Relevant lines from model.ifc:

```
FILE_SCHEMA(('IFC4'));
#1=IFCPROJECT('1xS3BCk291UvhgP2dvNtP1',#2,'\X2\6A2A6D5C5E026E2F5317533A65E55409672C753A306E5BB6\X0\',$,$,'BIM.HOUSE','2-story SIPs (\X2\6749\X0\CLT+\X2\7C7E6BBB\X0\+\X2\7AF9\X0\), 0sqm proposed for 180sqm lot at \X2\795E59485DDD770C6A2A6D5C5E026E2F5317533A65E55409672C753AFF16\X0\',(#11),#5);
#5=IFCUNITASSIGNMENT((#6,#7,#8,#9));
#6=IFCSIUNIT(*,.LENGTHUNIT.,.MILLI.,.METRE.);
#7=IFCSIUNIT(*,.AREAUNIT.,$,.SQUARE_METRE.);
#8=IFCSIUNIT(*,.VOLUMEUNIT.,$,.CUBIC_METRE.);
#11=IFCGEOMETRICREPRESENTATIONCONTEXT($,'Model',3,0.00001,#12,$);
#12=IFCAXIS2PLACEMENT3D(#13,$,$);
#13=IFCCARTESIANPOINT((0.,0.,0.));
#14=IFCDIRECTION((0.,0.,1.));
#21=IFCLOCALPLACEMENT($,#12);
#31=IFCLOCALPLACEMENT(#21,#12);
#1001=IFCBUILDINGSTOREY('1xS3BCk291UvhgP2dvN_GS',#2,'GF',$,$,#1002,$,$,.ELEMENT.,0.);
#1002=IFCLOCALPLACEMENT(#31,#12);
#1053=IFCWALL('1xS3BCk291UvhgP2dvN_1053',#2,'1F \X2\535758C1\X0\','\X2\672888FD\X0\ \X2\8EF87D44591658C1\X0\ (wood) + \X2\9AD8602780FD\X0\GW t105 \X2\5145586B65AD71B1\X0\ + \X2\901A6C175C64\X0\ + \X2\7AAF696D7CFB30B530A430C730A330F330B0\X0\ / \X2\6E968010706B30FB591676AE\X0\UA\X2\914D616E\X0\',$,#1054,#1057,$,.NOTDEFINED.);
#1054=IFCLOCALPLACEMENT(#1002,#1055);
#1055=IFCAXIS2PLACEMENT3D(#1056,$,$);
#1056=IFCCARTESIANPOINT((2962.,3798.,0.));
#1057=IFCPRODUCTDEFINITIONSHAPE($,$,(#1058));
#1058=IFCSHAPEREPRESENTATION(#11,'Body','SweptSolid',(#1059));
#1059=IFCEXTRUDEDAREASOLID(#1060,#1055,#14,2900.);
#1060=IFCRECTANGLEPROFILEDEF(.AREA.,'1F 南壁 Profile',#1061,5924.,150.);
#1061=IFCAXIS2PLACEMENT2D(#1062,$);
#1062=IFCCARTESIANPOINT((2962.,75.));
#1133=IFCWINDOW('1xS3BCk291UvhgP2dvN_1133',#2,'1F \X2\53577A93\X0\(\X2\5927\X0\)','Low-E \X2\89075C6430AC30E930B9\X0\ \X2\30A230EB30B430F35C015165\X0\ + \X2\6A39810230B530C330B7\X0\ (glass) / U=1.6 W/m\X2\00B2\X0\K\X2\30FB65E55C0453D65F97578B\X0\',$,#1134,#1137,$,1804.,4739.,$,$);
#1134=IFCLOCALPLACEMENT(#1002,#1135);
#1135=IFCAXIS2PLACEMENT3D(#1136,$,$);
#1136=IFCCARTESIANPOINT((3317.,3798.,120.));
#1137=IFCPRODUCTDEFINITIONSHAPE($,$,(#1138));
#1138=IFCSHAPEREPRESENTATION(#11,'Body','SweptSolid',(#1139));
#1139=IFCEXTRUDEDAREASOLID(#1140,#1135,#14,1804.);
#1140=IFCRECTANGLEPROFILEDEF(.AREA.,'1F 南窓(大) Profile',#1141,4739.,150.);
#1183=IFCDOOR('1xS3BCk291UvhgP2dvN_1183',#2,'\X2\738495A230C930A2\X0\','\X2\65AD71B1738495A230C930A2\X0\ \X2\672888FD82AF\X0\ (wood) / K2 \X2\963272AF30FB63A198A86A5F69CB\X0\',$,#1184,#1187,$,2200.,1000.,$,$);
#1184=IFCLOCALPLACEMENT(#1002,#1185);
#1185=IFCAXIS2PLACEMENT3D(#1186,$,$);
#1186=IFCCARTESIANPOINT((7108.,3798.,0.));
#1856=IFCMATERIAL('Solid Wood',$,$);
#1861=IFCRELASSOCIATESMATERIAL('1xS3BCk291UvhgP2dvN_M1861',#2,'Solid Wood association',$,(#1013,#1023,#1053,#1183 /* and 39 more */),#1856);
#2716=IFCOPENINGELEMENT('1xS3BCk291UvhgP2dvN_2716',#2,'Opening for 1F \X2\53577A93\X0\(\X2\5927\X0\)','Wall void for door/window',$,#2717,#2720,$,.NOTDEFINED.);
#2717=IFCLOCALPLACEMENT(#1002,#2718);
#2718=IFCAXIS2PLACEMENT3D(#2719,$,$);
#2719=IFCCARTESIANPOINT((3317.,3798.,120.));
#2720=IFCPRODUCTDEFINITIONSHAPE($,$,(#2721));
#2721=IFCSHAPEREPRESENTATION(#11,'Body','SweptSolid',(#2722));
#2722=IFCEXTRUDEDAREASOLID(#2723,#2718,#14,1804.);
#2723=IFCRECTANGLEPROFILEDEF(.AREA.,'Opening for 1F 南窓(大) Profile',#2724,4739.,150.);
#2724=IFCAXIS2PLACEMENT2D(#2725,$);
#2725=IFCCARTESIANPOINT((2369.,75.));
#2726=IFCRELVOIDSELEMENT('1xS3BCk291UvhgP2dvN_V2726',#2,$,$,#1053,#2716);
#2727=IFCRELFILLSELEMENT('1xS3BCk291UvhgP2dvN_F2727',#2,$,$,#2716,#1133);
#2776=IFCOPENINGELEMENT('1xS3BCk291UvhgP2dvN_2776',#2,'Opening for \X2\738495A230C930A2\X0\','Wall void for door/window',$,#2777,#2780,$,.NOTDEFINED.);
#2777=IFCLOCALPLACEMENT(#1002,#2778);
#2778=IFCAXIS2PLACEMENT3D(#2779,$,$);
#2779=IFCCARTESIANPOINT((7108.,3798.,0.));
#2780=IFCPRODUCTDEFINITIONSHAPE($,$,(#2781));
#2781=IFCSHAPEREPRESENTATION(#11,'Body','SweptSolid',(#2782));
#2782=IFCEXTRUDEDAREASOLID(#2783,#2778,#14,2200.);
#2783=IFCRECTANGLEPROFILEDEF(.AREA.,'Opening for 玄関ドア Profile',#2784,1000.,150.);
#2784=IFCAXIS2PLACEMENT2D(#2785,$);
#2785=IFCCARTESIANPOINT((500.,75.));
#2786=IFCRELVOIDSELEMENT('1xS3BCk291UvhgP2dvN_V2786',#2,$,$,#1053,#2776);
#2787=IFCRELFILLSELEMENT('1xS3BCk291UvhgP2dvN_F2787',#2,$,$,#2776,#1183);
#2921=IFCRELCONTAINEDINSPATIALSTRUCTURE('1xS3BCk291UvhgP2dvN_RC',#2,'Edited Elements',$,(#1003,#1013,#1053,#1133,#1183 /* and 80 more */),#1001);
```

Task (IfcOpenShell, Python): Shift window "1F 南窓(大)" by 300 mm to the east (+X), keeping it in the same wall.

```python
import ifcopenshell
import ifcopenshell.api.geometry
import ifcopenshell.util.placement
import ifcopenshell.util.unit

model = ifcopenshell.open("model.ifc")
unit_scale = ifcopenshell.util.unit.calculate_unit_scale(model)

window = model.by_guid("1xS3BCk291UvhgP2dvN_1133")
opening = window.FillsVoids[0].RelatingOpeningElement
wall = opening.VoidsElements[0].RelatingBuildingElement

wall_matrix = ifcopenshell.util.placement.get_local_placement(wall.ObjectPlacement)
shift = wall_matrix[:3, 0] * 0.3 / unit_scale
before = ifcopenshell.util.placement.get_local_placement(window.ObjectPlacement)[:3, 3].copy()

# The window is not placed relative to its opening, so move both.
for product in (opening, window):
    matrix = ifcopenshell.util.placement.get_local_placement(product.ObjectPlacement)
    matrix[:3, 3] += shift
    ifcopenshell.api.geometry.edit_object_placement(model, product=product, matrix=matrix, is_si=False)

after = ifcopenshell.util.placement.get_local_placement(window.ObjectPlacement)[:3, 3]
print("window moved by", (after - before).round(3) + 0.0)

model.write("model_edited.ifc")
```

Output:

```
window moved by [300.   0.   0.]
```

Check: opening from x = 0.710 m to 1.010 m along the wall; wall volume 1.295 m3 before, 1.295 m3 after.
